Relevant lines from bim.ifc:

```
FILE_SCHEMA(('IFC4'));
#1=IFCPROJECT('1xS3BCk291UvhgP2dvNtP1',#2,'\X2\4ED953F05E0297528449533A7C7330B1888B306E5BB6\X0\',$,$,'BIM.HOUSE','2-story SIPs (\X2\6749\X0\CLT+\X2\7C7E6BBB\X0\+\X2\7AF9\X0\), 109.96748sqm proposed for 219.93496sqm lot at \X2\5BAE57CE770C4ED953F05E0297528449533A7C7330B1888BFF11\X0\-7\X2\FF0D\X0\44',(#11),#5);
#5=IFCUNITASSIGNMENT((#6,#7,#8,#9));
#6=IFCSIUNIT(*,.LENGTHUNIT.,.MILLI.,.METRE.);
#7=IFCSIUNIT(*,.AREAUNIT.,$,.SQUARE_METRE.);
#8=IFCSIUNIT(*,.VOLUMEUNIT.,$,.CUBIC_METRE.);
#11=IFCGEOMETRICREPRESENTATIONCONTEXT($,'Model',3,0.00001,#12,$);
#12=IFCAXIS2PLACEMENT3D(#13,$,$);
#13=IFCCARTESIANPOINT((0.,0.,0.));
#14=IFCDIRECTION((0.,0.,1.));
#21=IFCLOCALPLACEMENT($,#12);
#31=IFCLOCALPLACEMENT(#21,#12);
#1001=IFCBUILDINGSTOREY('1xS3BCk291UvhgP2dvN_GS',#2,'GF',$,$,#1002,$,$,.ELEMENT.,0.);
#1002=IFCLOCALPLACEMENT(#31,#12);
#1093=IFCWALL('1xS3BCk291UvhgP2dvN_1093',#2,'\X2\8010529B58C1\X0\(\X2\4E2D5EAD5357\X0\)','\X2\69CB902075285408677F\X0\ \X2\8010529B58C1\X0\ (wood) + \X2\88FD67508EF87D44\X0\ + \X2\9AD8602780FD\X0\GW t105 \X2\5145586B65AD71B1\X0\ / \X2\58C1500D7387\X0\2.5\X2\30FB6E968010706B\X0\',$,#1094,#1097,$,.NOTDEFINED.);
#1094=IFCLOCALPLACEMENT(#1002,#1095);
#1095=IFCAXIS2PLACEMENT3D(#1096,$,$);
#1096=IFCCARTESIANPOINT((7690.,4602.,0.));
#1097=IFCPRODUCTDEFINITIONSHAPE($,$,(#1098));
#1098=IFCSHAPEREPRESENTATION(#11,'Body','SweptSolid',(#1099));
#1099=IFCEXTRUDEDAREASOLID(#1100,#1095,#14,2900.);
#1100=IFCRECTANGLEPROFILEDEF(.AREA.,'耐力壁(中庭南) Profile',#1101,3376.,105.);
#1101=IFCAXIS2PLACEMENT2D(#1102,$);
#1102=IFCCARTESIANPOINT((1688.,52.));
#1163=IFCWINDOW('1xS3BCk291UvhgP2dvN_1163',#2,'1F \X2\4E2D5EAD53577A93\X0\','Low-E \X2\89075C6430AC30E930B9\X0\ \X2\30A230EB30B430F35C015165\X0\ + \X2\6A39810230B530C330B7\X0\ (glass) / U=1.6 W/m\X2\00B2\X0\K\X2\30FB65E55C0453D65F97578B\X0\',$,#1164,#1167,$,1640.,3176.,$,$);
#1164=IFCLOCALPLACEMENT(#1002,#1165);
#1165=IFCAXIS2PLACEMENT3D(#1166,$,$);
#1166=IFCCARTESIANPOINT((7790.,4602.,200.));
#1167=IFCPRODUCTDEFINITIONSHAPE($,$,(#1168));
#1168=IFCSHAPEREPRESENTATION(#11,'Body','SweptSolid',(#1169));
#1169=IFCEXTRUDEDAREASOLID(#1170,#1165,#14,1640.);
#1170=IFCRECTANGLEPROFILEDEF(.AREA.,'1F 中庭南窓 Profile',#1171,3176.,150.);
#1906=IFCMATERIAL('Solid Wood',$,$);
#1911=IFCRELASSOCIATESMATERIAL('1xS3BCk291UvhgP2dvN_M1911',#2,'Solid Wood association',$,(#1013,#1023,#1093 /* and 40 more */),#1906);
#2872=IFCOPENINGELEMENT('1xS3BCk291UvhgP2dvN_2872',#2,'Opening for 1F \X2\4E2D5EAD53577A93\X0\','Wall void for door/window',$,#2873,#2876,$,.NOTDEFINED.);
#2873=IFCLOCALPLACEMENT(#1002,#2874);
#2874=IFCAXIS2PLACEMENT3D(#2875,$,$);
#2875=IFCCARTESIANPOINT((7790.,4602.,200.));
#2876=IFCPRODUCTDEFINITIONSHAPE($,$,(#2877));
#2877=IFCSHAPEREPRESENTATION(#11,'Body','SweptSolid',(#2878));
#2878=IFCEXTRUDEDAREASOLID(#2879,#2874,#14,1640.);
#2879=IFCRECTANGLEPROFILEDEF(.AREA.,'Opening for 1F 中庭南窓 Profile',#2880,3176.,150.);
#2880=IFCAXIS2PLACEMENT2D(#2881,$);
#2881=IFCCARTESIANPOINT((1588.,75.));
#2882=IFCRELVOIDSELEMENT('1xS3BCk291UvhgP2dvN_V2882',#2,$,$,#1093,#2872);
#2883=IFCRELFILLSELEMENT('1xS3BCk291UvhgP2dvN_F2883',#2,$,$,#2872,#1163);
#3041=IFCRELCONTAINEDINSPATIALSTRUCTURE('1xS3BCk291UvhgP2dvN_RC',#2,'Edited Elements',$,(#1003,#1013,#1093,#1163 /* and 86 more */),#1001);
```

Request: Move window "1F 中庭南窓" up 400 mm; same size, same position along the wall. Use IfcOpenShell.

```python
import numpy as np
import ifcopenshell
import ifcopenshell.api.geometry
import ifcopenshell.util.placement
import ifcopenshell.util.unit

model = ifcopenshell.open("bim.ifc")
unit_scale = ifcopenshell.util.unit.calculate_unit_scale(model)

window = model.by_guid("1xS3BCk291UvhgP2dvN_1163")
opening = window.FillsVoids[0].RelatingOpeningElement
dz = 0.4 / unit_scale

shift = np.array([0.0, 0.0, dz])
# The window is not placed relative to its opening, so move both.
for product in (opening, window):
    matrix = ifcopenshell.util.placement.get_local_placement(product.ObjectPlacement)
    matrix[:3, 3] += shift
    ifcopenshell.api.geometry.edit_object_placement(model, product=product, matrix=matrix, is_si=False)

print(f"moved by {dz * unit_scale:+.3f} m")

model.write("bim_updated.ifc")
```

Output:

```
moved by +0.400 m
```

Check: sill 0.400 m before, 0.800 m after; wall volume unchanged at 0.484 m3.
